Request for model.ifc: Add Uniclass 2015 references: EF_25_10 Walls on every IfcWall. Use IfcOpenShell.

First a look at what the model holds.

```python
import ifcopenshell

model = ifcopenshell.open("model.ifc")
print(model.schema)
print("classifications:", [c.Name for c in model.by_type("IfcClassification")])
for ifc_class in ("IfcDoor", "IfcRoof", "IfcStair", "IfcWall", "IfcWindow"):
    print(ifc_class, len(model.by_type(ifc_class)))
```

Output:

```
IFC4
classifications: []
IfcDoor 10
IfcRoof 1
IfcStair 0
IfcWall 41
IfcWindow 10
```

```python
import ifcopenshell
import ifcopenshell.api.classification

model = ifcopenshell.open("model.ifc")

system = ifcopenshell.api.classification.add_classification(model, classification="Uniclass 2015")

codes = {
    "IfcWall": ("EF_25_10", "Walls"),
}
for ifc_class, (code, name) in codes.items():
    products = model.by_type(ifc_class)
    ifcopenshell.api.classification.add_reference(
        model, products=products, classification=system, identification=code, name=name
    )
    print(code, len(products))

model.write("model_v2.ifc")
```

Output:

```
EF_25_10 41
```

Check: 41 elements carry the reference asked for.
